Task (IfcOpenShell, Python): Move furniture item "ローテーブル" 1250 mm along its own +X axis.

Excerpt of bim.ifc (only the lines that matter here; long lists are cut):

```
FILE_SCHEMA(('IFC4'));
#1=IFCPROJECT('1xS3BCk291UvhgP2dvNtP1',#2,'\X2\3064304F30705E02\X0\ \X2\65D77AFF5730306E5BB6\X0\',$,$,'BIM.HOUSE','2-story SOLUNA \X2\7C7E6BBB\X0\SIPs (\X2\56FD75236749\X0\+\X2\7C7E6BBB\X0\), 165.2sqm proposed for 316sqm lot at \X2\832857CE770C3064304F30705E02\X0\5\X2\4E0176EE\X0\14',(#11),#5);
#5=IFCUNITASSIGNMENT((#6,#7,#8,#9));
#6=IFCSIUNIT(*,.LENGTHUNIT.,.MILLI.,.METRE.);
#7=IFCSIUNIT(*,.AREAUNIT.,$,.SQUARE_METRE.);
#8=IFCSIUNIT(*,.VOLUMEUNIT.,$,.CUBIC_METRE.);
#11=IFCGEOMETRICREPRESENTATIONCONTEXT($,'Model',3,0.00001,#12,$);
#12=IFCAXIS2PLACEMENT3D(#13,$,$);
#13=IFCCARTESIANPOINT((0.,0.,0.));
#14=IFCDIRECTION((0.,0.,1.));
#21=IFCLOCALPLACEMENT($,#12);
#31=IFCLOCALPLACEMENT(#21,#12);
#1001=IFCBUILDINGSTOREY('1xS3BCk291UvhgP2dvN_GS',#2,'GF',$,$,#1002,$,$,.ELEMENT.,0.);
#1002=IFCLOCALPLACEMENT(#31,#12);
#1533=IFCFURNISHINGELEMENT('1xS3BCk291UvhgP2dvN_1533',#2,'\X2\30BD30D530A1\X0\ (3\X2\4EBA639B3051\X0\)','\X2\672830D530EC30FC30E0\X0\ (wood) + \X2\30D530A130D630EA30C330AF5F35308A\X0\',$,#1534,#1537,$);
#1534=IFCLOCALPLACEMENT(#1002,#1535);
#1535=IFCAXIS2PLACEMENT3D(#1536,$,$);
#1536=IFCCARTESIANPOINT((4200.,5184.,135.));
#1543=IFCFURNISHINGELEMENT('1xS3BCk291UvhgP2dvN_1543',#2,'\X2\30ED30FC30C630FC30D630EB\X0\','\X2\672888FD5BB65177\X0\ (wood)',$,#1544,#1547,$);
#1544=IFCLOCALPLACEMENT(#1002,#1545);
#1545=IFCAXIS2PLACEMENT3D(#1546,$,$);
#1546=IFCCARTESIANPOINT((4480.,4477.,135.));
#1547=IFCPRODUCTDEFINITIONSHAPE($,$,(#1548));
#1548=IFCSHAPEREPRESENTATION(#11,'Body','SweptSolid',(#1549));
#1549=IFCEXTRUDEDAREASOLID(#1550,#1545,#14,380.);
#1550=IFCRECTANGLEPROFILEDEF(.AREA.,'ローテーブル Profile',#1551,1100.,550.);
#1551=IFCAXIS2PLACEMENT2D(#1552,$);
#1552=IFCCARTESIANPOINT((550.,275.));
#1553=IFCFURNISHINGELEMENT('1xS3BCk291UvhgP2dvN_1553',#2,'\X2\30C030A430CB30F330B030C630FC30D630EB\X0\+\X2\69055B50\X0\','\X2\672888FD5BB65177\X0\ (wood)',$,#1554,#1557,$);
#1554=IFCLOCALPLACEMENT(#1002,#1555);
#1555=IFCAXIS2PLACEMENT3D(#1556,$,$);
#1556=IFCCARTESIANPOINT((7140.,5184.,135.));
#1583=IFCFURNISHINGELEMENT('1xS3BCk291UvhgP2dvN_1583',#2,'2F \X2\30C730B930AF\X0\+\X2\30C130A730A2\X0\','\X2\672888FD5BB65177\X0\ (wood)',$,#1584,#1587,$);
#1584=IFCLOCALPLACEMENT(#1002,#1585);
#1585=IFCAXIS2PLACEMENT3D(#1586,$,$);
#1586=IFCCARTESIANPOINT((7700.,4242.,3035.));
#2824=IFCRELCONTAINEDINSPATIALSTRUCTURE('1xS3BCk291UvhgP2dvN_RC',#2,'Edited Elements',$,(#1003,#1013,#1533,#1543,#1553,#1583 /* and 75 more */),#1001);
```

```python
import ifcopenshell
import ifcopenshell.api.geometry
import ifcopenshell.util.placement
import ifcopenshell.util.unit

model = ifcopenshell.open("bim.ifc")
unit_scale = ifcopenshell.util.unit.calculate_unit_scale(model)

item = model.by_guid("1xS3BCk291UvhgP2dvN_1543")
matrix = ifcopenshell.util.placement.get_local_placement(item.ObjectPlacement)
matrix[:3, 3] += matrix[:3, 0] * 1.25 / unit_scale
ifcopenshell.api.geometry.edit_object_placement(model, product=item, matrix=matrix, is_si=False)

print(ifcopenshell.util.placement.get_local_placement(item.ObjectPlacement).round(3) + 0.0)

model.write("bim_edited.ifc")
```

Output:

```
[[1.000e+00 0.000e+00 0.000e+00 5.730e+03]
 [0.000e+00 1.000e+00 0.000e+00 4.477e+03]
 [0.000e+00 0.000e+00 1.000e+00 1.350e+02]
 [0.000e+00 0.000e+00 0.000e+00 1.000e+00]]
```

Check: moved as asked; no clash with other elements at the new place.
